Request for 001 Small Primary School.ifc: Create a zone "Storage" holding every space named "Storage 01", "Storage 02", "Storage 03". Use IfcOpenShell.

First a look at what the model holds.

```python
import ifcopenshell

model = ifcopenshell.open("001 Small Primary School.ifc")
print(model.schema)
seen = {}
for space in model.by_type("IfcSpace"):
    seen[space.LongName] = seen.get(space.LongName, 0) + 1
for name, count in sorted(seen.items(), key=str):
    print(count, "x", name)
print("zones:", [z.Name for z in model.by_type("IfcZone")][:20])
```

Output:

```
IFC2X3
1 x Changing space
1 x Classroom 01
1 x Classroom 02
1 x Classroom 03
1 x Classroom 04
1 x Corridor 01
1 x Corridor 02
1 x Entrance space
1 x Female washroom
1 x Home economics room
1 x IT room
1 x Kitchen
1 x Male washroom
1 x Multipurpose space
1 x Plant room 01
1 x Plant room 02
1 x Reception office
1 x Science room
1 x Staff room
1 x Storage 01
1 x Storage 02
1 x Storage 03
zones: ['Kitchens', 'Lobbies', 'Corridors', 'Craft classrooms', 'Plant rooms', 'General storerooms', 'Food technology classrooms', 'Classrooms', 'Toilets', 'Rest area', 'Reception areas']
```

```python
import ifcopenshell
import ifcopenshell.api.group
import ifcopenshell.api.root

model = ifcopenshell.open("001 Small Primary School.ifc")

names = {"Storage 01", "Storage 02", "Storage 03"}
spaces = [s for s in model.by_type("IfcSpace") if s.LongName in names]

zone = ifcopenshell.api.root.create_entity(model, ifc_class="IfcZone", name="Storage")
ifcopenshell.api.group.assign_group(model, products=spaces, group=zone)
print(len(spaces), "spaces in", zone.Name)

model.write("001 Small Primary School_edited.ifc")
```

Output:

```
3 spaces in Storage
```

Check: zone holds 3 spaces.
